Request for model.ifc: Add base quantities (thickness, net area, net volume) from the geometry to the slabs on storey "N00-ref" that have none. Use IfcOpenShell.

First a look at what the model holds.

```python
import ifcopenshell
import ifcopenshell.util.element
import ifcopenshell.util.unit

model = ifcopenshell.open("model.ifc")
print(model.schema)
for unit_type in ("LENGTHUNIT", "AREAUNIT", "VOLUMEUNIT"):
    print(unit_type, ifcopenshell.util.unit.calculate_unit_scale(model, unit_type))
storey = next(s for s in model.by_type("IfcBuildingStorey") if s.Name == "N00-ref")
slabs = [e for e in ifcopenshell.util.element.get_decomposition(storey) if e.is_a("IfcSlab")]
for e in sorted(slabs, key=lambda e: e.id()):
    print(e.id(), e.is_a(), e.Name, list(ifcopenshell.util.element.get_psets(e, qtos_only=True)), sep=" | ")
```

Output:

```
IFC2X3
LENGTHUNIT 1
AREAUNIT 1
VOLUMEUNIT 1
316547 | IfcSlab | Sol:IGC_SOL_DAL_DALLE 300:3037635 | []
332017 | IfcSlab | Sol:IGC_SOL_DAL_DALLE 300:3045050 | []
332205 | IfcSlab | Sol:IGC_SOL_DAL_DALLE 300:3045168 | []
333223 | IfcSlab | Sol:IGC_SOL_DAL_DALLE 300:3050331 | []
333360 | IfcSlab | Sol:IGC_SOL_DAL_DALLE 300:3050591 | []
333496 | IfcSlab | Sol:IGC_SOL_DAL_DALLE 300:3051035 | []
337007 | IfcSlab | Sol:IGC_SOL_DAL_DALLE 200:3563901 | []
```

```python
import ifcopenshell
import ifcopenshell.api.pset
import ifcopenshell.geom
import ifcopenshell.util.element
import ifcopenshell.util.shape
import ifcopenshell.util.unit

model = ifcopenshell.open("model.ifc")
unit_scale = ifcopenshell.util.unit.calculate_unit_scale(model)
area_scale = ifcopenshell.util.unit.calculate_unit_scale(model, "AREAUNIT")
volume_scale = ifcopenshell.util.unit.calculate_unit_scale(model, "VOLUMEUNIT")
settings = ifcopenshell.geom.settings()

storey = next(s for s in model.by_type("IfcBuildingStorey") if s.Name == "N00-ref")
slabs = [e for e in ifcopenshell.util.element.get_decomposition(storey) if e.is_a("IfcSlab")]

for e in sorted(slabs, key=lambda e: e.id()):
    if ifcopenshell.util.element.get_psets(e, qtos_only=True, should_inherit=False):
        continue
    # Geometry comes back in metres, in the element's own axes.
    shape = ifcopenshell.geom.create_shape(settings, e)
    values = {
        "Width": ifcopenshell.util.shape.get_z(shape.geometry) / unit_scale,
        "NetArea": ifcopenshell.util.shape.get_footprint_area(shape.geometry) / area_scale,
        "NetVolume": ifcopenshell.util.shape.get_volume(shape.geometry) / volume_scale,
    }
    qto = ifcopenshell.api.pset.add_qto(model, product=e, name="BaseQuantities")
    ifcopenshell.api.pset.edit_qto(model, qto=qto, properties=values)
    print(e.id(), {k: round(v, 3) for k, v in values.items()})

model.write("model_v2.ifc")
```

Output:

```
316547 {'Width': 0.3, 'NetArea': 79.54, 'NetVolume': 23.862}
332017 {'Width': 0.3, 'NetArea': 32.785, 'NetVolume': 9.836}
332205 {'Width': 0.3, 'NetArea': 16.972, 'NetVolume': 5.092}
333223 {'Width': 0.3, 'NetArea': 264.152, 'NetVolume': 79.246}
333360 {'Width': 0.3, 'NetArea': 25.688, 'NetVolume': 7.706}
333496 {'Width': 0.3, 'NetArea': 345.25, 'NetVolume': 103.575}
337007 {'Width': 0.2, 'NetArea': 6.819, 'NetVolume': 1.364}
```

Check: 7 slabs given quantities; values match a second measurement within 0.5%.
